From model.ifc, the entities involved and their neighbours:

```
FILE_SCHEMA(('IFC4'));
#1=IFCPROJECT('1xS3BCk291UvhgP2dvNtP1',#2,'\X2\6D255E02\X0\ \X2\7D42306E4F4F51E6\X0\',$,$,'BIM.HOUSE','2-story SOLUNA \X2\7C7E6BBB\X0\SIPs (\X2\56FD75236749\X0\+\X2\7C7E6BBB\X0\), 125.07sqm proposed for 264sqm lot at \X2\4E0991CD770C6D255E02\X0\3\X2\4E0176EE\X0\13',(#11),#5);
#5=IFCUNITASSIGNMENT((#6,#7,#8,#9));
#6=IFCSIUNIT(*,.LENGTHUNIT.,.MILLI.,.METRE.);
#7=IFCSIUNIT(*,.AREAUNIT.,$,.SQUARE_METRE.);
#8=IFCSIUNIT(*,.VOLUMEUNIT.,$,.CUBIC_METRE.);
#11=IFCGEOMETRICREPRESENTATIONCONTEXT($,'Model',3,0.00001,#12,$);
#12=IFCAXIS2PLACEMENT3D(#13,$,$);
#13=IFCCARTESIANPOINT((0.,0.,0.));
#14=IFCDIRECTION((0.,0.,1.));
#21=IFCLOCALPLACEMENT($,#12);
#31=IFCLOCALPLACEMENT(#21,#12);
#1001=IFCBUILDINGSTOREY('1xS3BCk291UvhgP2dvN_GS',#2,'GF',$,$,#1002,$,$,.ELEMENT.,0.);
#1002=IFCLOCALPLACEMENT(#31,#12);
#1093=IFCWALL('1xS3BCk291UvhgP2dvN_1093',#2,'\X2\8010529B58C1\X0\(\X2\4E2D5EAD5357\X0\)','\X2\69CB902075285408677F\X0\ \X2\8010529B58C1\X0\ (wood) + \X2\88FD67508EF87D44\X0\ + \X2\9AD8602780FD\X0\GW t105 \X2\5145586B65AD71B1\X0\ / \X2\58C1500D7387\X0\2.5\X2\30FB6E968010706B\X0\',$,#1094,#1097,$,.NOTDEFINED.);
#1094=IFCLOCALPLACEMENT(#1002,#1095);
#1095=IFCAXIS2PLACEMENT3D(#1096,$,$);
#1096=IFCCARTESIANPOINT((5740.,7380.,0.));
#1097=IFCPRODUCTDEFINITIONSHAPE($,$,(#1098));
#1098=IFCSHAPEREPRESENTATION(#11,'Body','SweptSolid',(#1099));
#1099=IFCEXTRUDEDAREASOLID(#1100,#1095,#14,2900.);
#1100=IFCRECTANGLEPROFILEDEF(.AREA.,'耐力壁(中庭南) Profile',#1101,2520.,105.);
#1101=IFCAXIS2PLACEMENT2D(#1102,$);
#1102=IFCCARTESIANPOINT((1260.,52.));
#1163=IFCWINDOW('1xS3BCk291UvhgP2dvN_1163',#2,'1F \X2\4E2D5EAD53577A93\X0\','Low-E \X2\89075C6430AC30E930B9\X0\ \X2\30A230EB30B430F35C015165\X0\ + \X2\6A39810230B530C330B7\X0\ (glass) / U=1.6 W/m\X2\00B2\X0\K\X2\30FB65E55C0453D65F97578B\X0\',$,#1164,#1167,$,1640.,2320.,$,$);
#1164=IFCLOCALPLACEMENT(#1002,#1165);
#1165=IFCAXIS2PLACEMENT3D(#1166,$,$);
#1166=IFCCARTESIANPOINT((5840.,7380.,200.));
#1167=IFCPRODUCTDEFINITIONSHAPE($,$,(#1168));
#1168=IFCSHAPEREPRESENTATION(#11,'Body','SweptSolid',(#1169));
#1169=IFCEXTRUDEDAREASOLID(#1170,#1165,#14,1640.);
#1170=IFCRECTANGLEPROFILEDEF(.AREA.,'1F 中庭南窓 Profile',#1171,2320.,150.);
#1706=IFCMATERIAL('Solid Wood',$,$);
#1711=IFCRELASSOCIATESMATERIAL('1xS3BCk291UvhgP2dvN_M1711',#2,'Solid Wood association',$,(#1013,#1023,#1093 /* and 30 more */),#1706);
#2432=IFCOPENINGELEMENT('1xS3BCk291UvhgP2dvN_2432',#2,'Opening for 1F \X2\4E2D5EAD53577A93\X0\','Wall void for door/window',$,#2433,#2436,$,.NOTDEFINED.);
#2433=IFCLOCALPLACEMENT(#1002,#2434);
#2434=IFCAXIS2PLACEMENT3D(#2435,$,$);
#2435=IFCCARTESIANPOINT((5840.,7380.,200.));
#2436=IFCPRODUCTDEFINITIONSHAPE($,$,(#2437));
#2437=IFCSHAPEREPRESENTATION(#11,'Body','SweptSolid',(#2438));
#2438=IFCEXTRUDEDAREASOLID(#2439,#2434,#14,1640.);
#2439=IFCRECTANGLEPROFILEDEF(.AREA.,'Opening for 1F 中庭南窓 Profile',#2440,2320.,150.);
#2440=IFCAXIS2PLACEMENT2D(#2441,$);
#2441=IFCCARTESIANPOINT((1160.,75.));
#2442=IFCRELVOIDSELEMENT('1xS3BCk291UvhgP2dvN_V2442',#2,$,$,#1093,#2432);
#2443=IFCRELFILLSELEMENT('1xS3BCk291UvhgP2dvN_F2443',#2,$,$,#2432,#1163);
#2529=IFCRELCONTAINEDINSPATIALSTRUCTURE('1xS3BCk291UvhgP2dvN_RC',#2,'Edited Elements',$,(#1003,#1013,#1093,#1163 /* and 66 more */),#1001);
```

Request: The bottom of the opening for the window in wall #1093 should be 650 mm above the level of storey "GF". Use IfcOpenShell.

```python
import numpy as np
import ifcopenshell
import ifcopenshell.api.geometry
import ifcopenshell.geom
import ifcopenshell.util.element
import ifcopenshell.util.placement
import ifcopenshell.util.shape
import ifcopenshell.util.unit

model = ifcopenshell.open("model.ifc")
unit_scale = ifcopenshell.util.unit.calculate_unit_scale(model)

window = model.by_guid("1xS3BCk291UvhgP2dvN_1163")
opening = window.FillsVoids[0].RelatingOpeningElement
storey = ifcopenshell.util.element.get_container(window, ifc_class="IfcBuildingStorey")
level = ifcopenshell.util.placement.get_local_placement(storey.ObjectPlacement)[2, 3]

# The opening's origin need not be at the sill, so measure its lowest point.
shape = ifcopenshell.geom.create_shape(ifcopenshell.geom.settings(), opening)
bottom = ifcopenshell.util.shape.get_shape_bottom_elevation(shape, shape.geometry) / unit_scale
dz = level + 650.0 - bottom

shift = np.array([0.0, 0.0, dz])
# The window is not placed relative to its opening, so move both.
for product in (opening, window):
    matrix = ifcopenshell.util.placement.get_local_placement(product.ObjectPlacement)
    matrix[:3, 3] += shift
    ifcopenshell.api.geometry.edit_object_placement(model, product=product, matrix=matrix, is_si=False)

print(f"moved by {dz * unit_scale:+.3f} m")

model.write("model_v2.ifc")
```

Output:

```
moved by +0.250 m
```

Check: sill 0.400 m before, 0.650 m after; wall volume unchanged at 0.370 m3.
